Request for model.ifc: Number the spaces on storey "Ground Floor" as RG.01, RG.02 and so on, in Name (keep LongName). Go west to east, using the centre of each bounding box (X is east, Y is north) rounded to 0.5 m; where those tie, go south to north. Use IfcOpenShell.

First a look at what the model holds.

```python
import ifcopenshell
import ifcopenshell.util.element
import ifcopenshell.util.placement

model = ifcopenshell.open("model.ifc")
print(model.schema)
storey = next(s for s in model.by_type("IfcBuildingStorey") if s.Name == "Ground Floor")
spaces = [e for e in ifcopenshell.util.element.get_decomposition(storey) if e.is_a("IfcSpace")]
for e in sorted(spaces, key=lambda e: e.id()):
    origin = ifcopenshell.util.placement.get_local_placement(e.ObjectPlacement)[:3, 3]
    print(e.id(), e.Name, e.LongName, origin.round(2) + 0.0, sep=" | ")
```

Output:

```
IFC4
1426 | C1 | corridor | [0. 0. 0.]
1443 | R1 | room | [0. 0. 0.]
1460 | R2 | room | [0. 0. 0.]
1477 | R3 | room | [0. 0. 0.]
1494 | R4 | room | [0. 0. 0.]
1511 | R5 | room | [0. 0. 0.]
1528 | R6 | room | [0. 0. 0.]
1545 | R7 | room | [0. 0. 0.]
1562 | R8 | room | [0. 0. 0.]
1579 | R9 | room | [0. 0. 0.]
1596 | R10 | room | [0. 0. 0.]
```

```python
import ifcopenshell
import ifcopenshell.geom
import ifcopenshell.util.element
import ifcopenshell.util.shape

model = ifcopenshell.open("model.ifc")
settings = ifcopenshell.geom.settings()
settings.set("use-world-coords", True)


def centre(element):
    shape = ifcopenshell.geom.create_shape(settings, element)
    return ifcopenshell.util.shape.get_bbox_centroid(shape.geometry)


storey = next(s for s in model.by_type("IfcBuildingStorey") if s.Name == "Ground Floor")
spaces = [e for e in ifcopenshell.util.element.get_decomposition(storey) if e.is_a("IfcSpace")]

# Insertion points can sit at a corner or the storey origin, so sort by the geometry (in metres).
centres = {e: centre(e) for e in spaces}
spaces.sort(key=lambda e: (round(centres[e][0] / 0.5), centres[e][1]))

for i, e in enumerate(spaces, start=1):
    number = f"RG.{i:02d}"
    e.Name = number
    print(e.id(), number)

model.write("model_updated.ifc")
```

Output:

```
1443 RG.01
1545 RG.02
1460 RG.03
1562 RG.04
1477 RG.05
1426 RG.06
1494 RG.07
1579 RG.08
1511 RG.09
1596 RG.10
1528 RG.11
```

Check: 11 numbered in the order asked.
